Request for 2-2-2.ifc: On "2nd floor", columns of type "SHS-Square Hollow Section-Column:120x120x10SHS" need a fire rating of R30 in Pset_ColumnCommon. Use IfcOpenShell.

First a look at what the model holds.

```python
import ifcopenshell
import ifcopenshell.util.element

model = ifcopenshell.open("2-2-2.ifc")
print(model.schema)
storey = next(s for s in model.by_type("IfcBuildingStorey") if s.Name == "2nd floor")
columns = [e for e in ifcopenshell.util.element.get_decomposition(storey) if e.is_a("IfcColumn")]
seen = {}
for e in columns:
    element_type = ifcopenshell.util.element.get_type(e)
    key = (element_type.Name if element_type != e and element_type else None, ifcopenshell.util.element.get_pset(e, "Pset_ColumnCommon", "FireRating"))
    seen[key] = seen.get(key, 0) + 1
for (name, value), count in sorted(seen.items(), key=str):
    print(count, "x", name, "|", value)
```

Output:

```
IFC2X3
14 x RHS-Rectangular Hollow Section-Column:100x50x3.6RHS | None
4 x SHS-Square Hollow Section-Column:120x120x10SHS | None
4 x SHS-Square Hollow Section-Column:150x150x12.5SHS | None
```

```python
import ifcopenshell
import ifcopenshell.api.pset
import ifcopenshell.util.element

model = ifcopenshell.open("2-2-2.ifc")

storey = next(s for s in model.by_type("IfcBuildingStorey") if s.Name == "2nd floor")
columns = [e for e in ifcopenshell.util.element.get_decomposition(storey) if e.is_a("IfcColumn")]

count = 0
for e in columns:
    element_type = ifcopenshell.util.element.get_type(e)
    if element_type in (None, e) or element_type.Name != "SHS-Square Hollow Section-Column:120x120x10SHS":
        continue
    # add_pset returns the element's existing set when there is one.
    pset = ifcopenshell.api.pset.add_pset(model, product=e, name="Pset_ColumnCommon")
    ifcopenshell.api.pset.edit_pset(model, pset=pset, properties={"FireRating": "R30"})
    count += 1

print(count, "columns updated")

model.write("2-2-2-out.ifc")
```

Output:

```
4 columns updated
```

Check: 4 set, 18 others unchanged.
